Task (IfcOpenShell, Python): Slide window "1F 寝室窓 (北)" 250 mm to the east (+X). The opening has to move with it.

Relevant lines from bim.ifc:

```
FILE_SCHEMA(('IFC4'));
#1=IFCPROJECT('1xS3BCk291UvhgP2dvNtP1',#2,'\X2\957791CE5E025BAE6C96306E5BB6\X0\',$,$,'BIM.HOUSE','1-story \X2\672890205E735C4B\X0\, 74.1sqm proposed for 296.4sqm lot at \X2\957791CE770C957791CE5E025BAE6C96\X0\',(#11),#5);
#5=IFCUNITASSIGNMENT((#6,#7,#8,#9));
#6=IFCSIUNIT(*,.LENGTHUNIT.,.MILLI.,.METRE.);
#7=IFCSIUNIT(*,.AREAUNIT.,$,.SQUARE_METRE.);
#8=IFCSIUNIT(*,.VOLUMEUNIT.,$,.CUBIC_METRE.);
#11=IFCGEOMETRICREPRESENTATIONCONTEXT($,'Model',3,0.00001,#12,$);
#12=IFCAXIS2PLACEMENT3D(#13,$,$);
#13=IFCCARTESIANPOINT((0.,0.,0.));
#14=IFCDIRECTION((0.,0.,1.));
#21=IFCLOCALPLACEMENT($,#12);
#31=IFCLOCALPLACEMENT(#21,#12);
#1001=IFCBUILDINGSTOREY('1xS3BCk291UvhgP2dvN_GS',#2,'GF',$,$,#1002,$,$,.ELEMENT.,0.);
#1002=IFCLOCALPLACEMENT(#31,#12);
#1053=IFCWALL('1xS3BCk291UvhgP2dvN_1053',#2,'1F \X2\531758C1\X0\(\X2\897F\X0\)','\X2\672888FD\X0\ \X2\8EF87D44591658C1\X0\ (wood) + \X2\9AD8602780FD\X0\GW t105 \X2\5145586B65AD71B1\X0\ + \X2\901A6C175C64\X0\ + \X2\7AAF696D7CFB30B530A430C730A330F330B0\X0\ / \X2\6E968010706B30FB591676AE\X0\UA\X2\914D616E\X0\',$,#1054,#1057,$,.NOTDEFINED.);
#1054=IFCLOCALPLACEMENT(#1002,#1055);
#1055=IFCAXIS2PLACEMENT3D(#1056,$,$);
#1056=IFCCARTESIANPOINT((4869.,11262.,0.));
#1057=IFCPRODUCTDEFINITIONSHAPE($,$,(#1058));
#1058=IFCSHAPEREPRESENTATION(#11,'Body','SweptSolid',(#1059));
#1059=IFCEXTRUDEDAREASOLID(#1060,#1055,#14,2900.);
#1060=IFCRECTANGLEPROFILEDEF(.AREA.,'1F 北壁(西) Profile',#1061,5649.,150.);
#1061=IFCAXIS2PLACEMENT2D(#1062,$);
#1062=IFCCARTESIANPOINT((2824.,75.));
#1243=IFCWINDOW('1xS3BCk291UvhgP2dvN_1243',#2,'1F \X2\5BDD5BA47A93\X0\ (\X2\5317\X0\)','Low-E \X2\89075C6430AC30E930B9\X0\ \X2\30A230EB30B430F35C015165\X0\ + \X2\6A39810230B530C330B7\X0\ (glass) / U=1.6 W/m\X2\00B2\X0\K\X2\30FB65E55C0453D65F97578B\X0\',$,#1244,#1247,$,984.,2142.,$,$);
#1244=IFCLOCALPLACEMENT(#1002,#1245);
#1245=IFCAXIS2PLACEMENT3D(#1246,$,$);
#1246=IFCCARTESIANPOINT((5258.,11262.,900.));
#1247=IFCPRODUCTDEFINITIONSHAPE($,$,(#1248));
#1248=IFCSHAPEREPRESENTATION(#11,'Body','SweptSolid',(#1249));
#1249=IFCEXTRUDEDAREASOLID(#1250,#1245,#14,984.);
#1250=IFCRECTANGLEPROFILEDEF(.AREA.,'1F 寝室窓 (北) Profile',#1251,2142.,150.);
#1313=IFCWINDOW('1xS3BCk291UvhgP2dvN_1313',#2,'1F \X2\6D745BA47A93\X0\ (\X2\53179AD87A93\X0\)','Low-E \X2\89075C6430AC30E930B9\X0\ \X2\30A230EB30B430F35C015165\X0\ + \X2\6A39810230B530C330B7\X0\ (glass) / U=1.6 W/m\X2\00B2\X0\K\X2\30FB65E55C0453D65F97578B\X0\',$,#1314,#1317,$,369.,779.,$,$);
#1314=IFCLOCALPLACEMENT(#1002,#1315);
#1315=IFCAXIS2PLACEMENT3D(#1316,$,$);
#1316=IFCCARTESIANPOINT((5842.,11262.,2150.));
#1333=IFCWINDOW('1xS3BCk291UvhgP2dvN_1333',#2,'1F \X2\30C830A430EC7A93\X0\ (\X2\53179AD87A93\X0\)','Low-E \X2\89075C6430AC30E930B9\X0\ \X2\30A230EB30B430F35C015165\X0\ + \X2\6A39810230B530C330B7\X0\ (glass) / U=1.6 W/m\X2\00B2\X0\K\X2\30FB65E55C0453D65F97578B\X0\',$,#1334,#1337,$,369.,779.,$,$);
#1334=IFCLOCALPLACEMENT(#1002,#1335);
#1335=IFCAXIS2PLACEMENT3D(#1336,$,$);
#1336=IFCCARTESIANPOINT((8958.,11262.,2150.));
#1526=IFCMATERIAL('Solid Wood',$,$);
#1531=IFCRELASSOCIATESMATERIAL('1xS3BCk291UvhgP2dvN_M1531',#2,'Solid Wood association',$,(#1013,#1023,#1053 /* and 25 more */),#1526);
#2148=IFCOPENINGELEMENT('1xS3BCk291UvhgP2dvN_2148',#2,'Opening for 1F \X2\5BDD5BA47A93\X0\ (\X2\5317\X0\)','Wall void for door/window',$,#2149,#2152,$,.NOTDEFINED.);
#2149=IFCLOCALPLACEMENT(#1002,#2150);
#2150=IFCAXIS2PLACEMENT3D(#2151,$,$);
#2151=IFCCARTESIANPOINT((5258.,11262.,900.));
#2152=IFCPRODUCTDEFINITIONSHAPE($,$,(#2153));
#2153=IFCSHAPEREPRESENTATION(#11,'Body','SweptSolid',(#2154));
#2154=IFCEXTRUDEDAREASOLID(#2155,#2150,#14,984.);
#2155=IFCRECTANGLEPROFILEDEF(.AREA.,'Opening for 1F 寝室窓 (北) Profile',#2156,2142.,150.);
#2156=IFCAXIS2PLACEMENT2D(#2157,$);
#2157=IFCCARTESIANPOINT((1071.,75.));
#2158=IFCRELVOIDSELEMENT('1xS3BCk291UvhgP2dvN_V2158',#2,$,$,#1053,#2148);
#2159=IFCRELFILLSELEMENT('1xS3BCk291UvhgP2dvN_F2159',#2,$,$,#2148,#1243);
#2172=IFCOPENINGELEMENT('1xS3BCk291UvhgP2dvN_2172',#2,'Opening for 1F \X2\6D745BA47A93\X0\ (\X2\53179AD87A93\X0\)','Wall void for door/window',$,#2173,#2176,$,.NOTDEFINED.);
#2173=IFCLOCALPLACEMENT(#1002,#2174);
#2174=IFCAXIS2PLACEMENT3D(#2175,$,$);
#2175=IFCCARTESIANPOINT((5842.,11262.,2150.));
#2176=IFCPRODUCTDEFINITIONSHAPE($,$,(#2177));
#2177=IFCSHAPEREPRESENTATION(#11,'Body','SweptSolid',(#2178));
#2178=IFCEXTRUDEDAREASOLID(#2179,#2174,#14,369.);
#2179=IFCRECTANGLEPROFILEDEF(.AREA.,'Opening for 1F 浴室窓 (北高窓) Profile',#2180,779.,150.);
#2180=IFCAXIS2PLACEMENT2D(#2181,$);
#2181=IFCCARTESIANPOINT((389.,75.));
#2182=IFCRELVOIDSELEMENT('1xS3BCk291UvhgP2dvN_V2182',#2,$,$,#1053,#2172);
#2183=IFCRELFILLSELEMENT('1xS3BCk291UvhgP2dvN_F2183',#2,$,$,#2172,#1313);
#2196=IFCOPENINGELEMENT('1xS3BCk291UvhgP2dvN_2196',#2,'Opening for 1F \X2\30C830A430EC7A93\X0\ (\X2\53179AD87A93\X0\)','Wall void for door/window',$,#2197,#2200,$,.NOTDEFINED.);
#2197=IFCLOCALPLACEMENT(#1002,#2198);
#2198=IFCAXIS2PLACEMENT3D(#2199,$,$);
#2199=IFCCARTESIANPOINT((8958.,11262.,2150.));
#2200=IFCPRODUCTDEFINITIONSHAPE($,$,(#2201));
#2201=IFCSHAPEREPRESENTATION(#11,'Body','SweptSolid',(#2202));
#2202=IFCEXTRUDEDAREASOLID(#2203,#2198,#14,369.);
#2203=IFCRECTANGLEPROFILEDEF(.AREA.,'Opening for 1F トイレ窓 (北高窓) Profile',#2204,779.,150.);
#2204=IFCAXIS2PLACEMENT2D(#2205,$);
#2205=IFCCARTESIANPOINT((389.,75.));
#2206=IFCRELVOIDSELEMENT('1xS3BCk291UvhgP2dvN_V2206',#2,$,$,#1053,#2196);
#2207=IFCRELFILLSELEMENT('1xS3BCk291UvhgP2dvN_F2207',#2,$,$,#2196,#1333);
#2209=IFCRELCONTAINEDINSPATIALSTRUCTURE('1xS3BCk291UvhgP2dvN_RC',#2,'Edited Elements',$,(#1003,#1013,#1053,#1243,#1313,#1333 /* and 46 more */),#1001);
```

```python
import ifcopenshell
import ifcopenshell.api.geometry
import ifcopenshell.util.placement

model = ifcopenshell.open("bim.ifc")

window = model.by_guid("1xS3BCk291UvhgP2dvN_1243")
opening = window.FillsVoids[0].RelatingOpeningElement
wall = opening.VoidsElements[0].RelatingBuildingElement

wall_matrix = ifcopenshell.util.placement.get_local_placement(wall.ObjectPlacement)
shift = wall_matrix[:3, 0] * 250.0
before = ifcopenshell.util.placement.get_local_placement(window.ObjectPlacement)[:3, 3].copy()

# The window is not placed relative to its opening, so move both.
for product in (opening, window):
    matrix = ifcopenshell.util.placement.get_local_placement(product.ObjectPlacement)
    matrix[:3, 3] += shift
    ifcopenshell.api.geometry.edit_object_placement(model, product=product, matrix=matrix, is_si=False)

after = ifcopenshell.util.placement.get_local_placement(window.ObjectPlacement)[:3, 3]
print("window moved by", (after - before).round(3) + 0.0)

model.write("bim_updated.ifc")
```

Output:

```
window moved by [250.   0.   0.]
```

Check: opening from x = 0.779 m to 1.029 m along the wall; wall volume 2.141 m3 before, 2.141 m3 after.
